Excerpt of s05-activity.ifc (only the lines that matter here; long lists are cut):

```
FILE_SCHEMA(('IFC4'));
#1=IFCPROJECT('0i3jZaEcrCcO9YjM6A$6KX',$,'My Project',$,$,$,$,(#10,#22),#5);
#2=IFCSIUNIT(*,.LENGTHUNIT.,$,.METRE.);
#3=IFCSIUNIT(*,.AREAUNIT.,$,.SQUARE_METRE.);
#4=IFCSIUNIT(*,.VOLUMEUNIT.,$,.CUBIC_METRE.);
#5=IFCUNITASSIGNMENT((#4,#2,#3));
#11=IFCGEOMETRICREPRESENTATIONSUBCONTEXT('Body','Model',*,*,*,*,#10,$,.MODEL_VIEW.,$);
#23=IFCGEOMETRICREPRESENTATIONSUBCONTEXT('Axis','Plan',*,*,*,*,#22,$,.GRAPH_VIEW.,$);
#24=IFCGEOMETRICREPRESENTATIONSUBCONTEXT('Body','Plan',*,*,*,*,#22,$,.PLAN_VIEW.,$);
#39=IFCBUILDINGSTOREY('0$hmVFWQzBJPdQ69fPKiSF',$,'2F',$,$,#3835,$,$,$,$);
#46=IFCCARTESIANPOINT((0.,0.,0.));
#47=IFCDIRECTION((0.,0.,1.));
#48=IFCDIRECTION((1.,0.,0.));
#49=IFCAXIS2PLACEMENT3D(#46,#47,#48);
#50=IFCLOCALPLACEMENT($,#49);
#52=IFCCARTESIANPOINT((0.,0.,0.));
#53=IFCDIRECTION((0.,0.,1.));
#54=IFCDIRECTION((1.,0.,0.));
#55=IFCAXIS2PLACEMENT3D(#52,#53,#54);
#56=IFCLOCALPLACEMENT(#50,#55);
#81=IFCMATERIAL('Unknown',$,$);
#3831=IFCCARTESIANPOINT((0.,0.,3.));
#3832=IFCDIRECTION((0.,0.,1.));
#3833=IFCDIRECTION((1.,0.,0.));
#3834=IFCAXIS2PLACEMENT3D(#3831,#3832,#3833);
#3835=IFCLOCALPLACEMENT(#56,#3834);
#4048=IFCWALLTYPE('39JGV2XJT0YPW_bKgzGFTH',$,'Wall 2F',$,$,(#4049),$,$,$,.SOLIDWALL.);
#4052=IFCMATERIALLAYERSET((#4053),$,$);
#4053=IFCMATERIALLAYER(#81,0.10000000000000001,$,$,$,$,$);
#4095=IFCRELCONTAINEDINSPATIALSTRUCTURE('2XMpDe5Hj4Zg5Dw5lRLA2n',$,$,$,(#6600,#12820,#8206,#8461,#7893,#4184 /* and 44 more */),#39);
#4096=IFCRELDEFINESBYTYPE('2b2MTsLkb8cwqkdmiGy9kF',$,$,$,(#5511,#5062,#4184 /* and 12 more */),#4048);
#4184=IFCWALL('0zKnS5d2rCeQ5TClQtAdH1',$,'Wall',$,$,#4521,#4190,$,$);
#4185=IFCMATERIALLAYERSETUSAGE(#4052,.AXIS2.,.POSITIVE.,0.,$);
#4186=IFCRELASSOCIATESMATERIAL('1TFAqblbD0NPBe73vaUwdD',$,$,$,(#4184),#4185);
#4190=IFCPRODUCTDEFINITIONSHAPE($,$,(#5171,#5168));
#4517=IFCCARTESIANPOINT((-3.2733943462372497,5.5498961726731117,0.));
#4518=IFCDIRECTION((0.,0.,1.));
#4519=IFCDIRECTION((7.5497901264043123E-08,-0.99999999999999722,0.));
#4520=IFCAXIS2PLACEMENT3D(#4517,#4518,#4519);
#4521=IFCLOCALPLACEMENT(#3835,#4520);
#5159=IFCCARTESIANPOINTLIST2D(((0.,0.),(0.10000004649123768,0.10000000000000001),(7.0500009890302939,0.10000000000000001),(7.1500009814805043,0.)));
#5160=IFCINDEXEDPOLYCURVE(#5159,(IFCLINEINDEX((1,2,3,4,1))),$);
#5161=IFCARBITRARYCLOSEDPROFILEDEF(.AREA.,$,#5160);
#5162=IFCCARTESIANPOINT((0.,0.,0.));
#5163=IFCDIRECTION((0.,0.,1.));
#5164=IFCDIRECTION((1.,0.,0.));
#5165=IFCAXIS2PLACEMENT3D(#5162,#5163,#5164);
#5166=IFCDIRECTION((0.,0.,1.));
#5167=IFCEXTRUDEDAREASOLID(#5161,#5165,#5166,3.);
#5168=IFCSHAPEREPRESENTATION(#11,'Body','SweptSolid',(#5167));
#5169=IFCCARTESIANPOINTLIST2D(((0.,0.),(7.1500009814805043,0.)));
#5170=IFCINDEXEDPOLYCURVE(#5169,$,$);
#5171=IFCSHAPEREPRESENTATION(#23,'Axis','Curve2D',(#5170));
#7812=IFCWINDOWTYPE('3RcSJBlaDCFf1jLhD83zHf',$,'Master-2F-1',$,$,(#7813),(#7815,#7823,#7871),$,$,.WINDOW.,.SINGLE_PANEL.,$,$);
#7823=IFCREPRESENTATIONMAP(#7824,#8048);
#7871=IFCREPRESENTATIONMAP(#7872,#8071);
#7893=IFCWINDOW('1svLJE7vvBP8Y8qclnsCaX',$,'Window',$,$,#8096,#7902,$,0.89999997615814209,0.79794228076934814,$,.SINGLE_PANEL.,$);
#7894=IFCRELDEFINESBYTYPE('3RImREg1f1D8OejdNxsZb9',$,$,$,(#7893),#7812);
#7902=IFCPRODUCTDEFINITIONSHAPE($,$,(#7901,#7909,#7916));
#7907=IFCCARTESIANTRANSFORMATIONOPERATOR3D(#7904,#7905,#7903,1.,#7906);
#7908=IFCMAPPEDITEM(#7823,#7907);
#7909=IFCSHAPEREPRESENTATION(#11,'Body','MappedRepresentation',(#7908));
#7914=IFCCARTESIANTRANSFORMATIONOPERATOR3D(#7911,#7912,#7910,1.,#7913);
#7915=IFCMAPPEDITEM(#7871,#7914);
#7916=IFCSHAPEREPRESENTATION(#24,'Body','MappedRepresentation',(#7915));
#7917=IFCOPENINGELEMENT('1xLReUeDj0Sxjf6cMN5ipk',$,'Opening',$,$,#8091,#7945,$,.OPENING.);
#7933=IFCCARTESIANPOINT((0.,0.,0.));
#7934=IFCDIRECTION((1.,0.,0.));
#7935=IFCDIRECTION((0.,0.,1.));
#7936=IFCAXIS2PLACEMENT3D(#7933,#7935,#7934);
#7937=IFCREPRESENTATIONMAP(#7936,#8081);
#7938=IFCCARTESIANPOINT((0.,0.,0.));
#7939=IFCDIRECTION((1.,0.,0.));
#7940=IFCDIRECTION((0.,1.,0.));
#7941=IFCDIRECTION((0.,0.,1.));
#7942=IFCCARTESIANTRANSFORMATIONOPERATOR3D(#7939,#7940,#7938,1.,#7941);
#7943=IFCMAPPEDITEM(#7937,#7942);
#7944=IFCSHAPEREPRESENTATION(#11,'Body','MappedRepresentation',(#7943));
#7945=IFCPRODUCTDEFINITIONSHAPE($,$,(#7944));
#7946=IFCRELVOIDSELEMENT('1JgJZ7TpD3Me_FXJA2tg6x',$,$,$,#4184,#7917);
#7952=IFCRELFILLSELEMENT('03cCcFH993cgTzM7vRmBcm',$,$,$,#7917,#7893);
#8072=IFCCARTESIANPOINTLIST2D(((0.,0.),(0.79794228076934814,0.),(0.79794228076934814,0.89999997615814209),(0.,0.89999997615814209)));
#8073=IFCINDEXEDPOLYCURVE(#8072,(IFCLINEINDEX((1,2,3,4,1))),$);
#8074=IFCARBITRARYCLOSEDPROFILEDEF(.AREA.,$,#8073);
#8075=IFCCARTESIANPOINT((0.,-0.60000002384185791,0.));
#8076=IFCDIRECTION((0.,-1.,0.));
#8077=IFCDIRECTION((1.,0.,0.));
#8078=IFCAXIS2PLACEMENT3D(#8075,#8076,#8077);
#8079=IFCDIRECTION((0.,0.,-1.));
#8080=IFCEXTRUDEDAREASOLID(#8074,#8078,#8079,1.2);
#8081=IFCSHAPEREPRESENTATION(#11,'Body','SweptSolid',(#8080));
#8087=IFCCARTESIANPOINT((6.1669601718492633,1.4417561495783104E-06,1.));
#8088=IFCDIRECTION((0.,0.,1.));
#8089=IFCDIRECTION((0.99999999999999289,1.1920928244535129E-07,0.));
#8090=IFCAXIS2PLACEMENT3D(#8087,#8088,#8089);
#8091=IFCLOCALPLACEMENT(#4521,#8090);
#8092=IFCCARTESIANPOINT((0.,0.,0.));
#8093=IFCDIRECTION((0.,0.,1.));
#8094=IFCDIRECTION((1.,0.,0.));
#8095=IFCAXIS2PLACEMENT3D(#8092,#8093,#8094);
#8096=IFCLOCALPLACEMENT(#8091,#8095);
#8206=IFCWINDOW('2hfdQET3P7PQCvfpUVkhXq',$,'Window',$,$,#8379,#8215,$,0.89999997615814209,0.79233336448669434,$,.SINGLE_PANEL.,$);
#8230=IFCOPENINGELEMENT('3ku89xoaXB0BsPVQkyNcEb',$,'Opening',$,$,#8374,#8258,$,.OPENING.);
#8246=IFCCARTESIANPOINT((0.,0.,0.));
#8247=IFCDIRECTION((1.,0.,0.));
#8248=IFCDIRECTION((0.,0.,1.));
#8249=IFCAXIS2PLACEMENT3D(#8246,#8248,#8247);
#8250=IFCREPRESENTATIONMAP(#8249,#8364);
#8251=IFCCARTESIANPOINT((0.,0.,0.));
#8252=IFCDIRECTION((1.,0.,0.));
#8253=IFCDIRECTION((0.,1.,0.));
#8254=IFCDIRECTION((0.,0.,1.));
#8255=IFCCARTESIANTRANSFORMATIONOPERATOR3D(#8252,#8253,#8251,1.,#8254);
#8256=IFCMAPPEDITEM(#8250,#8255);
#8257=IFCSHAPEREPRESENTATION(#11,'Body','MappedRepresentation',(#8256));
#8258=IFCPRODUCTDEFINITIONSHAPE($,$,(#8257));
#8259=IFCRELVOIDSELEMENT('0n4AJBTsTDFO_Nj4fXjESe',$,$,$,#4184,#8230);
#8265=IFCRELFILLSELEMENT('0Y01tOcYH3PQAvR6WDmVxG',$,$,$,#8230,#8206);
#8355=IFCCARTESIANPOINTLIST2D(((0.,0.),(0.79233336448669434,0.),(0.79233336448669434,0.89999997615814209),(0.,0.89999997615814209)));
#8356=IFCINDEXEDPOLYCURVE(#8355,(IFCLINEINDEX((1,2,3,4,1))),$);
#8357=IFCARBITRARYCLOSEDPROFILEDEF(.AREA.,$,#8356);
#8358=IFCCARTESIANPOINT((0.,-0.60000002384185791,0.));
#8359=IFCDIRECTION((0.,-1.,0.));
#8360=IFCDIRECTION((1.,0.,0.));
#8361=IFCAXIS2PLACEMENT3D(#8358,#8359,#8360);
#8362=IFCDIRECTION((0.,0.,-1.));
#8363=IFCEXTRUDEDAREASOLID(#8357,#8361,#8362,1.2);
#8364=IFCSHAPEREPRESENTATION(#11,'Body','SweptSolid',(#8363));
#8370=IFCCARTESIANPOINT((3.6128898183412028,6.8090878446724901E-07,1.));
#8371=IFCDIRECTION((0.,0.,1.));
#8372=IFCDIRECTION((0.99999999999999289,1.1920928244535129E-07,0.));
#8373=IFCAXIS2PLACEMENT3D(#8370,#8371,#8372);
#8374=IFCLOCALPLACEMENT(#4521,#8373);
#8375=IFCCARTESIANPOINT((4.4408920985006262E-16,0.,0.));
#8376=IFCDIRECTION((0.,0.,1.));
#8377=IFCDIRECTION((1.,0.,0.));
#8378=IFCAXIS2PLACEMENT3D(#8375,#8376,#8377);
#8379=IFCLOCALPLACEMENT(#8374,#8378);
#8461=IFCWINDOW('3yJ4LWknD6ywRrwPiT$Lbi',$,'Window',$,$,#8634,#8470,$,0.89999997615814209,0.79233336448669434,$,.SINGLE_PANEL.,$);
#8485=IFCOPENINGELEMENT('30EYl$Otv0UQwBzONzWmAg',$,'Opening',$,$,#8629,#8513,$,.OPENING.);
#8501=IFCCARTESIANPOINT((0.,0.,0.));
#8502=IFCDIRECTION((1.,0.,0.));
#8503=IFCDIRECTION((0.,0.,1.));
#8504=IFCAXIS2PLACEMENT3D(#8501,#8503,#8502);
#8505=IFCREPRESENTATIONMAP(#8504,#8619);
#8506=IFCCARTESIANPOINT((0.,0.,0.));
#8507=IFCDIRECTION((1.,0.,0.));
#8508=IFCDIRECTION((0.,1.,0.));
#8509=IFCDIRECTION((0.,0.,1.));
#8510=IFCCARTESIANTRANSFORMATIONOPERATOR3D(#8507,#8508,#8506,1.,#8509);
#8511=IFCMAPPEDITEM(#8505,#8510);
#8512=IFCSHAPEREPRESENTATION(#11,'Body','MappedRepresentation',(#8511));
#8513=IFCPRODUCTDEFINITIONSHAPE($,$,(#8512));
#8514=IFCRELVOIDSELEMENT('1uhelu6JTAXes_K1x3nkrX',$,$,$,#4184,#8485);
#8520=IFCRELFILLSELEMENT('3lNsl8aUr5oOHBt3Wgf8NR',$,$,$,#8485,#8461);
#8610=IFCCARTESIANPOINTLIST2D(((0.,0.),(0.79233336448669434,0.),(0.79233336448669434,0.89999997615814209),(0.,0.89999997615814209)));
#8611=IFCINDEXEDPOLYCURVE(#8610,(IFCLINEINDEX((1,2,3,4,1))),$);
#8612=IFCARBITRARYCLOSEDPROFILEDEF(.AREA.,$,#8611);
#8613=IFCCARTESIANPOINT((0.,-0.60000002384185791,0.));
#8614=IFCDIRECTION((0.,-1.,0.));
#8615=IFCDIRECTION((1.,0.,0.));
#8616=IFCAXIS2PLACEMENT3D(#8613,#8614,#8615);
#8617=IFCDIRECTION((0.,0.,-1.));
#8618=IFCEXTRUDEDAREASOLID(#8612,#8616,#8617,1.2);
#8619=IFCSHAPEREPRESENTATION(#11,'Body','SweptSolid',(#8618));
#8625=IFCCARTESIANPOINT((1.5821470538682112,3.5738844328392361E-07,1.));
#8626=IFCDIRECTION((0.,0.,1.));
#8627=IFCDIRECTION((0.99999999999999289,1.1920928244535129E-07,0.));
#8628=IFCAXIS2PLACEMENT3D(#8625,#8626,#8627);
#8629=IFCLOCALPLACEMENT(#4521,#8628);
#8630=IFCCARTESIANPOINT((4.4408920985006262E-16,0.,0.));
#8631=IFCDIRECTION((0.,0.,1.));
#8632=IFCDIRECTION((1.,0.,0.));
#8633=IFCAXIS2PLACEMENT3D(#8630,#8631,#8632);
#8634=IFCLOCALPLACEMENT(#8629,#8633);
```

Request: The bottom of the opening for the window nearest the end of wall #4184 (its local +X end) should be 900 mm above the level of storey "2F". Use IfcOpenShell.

```python
import numpy as np
import ifcopenshell
import ifcopenshell.api.geometry
import ifcopenshell.geom
import ifcopenshell.util.element
import ifcopenshell.util.placement
import ifcopenshell.util.shape
import ifcopenshell.util.unit

model = ifcopenshell.open("s05-activity.ifc")
unit_scale = ifcopenshell.util.unit.calculate_unit_scale(model)

window = model.by_guid("1svLJE7vvBP8Y8qclnsCaX")
opening = window.FillsVoids[0].RelatingOpeningElement
storey = ifcopenshell.util.element.get_container(window, ifc_class="IfcBuildingStorey")
level = ifcopenshell.util.placement.get_local_placement(storey.ObjectPlacement)[2, 3]

# The opening's origin need not be at the sill, so measure its lowest point.
shape = ifcopenshell.geom.create_shape(ifcopenshell.geom.settings(), opening)
bottom = ifcopenshell.util.shape.get_shape_bottom_elevation(shape, shape.geometry) / unit_scale
dz = level + 0.9 / unit_scale - bottom

shift = np.array([0.0, 0.0, dz])
# The window is placed relative to its opening, so it follows when the opening moves.
matrix = ifcopenshell.util.placement.get_local_placement(opening.ObjectPlacement)
matrix[:3, 3] += shift
ifcopenshell.api.geometry.edit_object_placement(
    model, product=opening, matrix=matrix, is_si=False, should_transform_children=True
)

print(f"moved by {dz * unit_scale:+.3f} m")

model.write("s05-activity_updated.ifc")
```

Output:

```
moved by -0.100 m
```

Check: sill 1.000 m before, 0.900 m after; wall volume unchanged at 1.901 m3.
